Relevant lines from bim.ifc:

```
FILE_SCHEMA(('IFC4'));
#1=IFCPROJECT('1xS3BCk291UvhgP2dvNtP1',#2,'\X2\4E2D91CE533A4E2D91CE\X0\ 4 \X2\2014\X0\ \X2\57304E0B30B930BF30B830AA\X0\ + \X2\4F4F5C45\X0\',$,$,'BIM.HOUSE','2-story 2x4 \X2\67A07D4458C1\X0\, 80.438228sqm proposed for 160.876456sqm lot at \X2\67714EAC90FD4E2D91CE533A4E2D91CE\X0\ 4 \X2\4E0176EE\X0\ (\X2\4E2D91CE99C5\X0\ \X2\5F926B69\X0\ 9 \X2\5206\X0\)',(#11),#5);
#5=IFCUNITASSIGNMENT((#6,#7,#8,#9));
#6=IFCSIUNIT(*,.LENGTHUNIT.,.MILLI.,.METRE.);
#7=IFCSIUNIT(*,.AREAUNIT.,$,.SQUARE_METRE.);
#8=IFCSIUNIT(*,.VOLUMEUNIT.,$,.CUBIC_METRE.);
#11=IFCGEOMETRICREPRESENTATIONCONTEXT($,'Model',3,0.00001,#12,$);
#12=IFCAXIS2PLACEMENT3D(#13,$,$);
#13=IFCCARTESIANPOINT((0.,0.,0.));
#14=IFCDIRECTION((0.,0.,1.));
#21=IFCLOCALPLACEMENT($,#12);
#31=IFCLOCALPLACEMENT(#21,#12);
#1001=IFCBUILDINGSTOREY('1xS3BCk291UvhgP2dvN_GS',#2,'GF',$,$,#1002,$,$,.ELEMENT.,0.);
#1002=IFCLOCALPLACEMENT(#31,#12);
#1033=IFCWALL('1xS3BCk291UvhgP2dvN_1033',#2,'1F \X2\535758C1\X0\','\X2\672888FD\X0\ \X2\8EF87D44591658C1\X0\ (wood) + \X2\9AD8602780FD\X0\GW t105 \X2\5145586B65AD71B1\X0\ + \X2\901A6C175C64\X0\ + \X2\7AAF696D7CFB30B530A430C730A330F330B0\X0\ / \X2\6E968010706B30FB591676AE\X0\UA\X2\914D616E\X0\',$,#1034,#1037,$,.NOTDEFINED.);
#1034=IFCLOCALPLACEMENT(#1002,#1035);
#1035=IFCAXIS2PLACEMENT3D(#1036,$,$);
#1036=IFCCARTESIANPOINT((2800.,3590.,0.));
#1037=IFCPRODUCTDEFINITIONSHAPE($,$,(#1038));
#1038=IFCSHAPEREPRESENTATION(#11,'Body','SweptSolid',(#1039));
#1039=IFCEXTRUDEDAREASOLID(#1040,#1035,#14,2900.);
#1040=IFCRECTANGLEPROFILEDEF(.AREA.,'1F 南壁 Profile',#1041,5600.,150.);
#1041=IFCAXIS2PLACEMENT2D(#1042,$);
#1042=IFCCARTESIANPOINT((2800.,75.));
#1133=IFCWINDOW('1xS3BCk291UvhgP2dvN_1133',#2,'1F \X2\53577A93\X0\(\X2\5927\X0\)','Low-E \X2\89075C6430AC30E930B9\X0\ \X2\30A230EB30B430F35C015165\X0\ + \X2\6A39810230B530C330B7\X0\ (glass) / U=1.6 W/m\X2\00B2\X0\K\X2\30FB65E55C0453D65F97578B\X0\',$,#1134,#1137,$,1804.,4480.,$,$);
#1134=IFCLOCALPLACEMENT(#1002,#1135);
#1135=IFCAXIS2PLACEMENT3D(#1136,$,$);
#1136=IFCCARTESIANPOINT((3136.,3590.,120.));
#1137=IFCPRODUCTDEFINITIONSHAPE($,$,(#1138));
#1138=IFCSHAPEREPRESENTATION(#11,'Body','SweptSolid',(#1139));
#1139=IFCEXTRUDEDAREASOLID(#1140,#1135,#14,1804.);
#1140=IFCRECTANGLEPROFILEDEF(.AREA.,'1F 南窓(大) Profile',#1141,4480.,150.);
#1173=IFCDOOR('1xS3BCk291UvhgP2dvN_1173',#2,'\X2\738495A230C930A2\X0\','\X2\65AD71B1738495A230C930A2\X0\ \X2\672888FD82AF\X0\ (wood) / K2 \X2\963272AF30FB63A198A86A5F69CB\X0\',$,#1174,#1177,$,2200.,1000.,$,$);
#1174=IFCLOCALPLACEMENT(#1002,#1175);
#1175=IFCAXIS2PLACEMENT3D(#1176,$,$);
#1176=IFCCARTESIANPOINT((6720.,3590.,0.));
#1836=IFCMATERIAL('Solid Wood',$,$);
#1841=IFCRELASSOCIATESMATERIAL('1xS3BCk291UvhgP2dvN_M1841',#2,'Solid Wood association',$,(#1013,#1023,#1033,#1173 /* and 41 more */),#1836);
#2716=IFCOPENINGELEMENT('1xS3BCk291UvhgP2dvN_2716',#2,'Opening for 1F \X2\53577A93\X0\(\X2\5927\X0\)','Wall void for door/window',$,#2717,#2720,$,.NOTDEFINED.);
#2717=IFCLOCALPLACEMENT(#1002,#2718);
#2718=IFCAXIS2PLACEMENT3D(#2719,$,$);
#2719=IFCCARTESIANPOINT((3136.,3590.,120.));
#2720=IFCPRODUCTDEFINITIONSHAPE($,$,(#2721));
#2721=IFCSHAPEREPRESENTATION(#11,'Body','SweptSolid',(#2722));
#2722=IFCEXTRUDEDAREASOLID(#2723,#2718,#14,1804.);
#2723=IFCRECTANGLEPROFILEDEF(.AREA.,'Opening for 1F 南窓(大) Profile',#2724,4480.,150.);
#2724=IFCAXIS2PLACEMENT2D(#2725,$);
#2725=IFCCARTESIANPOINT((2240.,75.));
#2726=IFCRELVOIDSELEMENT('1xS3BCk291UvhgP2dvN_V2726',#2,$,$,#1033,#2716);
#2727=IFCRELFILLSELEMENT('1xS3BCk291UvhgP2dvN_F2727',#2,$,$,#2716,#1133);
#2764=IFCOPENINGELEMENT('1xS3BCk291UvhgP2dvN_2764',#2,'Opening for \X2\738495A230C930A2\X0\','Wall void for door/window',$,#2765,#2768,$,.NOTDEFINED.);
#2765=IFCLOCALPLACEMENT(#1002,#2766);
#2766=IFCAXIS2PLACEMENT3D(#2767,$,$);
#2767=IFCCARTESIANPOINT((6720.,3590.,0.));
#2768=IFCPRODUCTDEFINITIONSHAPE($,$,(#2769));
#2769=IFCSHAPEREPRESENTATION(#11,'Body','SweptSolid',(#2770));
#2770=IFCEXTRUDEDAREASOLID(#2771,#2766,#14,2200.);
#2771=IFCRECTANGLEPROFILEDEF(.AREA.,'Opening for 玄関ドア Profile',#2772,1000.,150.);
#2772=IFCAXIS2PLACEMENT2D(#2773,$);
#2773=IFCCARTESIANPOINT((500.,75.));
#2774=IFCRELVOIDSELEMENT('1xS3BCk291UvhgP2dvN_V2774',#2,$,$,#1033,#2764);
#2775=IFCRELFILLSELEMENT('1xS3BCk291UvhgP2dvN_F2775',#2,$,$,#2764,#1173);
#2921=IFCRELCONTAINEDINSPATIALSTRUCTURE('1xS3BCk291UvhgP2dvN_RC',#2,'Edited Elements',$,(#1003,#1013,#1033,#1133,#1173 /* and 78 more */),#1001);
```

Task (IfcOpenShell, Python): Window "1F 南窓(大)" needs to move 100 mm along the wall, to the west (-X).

```python
import ifcopenshell
import ifcopenshell.api.geometry
import ifcopenshell.util.placement
import ifcopenshell.util.unit

model = ifcopenshell.open("bim.ifc")
unit_scale = ifcopenshell.util.unit.calculate_unit_scale(model)

window = model.by_id(1133)
opening = window.FillsVoids[0].RelatingOpeningElement
wall = opening.VoidsElements[0].RelatingBuildingElement

wall_matrix = ifcopenshell.util.placement.get_local_placement(wall.ObjectPlacement)
shift = wall_matrix[:3, 0] * -0.1 / unit_scale
before = ifcopenshell.util.placement.get_local_placement(window.ObjectPlacement)[:3, 3].copy()

# The window is not placed relative to its opening, so move both.
for product in (opening, window):
    matrix = ifcopenshell.util.placement.get_local_placement(product.ObjectPlacement)
    matrix[:3, 3] += shift
    ifcopenshell.api.geometry.edit_object_placement(model, product=product, matrix=matrix, is_si=False)

after = ifcopenshell.util.placement.get_local_placement(window.ObjectPlacement)[:3, 3]
print("window moved by", (after - before).round(3) + 0.0)

model.write("bim_edited.ifc")
```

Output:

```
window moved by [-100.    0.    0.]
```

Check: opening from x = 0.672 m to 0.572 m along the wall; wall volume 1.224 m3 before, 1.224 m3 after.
